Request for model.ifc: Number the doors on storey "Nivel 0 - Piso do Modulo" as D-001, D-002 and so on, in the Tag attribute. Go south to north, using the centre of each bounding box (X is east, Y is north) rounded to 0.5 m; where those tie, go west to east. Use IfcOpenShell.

First a look at what the model holds.

```python
import ifcopenshell
import ifcopenshell.util.element
import ifcopenshell.util.placement

model = ifcopenshell.open("model.ifc")
print(model.schema)
storey = next(s for s in model.by_type("IfcBuildingStorey") if s.Name == "Nivel 0 - Piso do Modulo")
doors = [e for e in ifcopenshell.util.element.get_decomposition(storey) if e.is_a("IfcDoor")]
for e in sorted(doors, key=lambda e: e.id()):
    origin = ifcopenshell.util.placement.get_local_placement(e.ObjectPlacement)[:3, 3]
    print(e.id(), e.Tag, e.Name, origin.round(2) + 0.0, sep=" | ")
```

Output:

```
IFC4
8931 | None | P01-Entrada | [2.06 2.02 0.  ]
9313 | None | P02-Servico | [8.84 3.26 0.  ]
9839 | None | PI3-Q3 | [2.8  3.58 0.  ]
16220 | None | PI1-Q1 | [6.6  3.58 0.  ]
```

```python
import ifcopenshell
import ifcopenshell.geom
import ifcopenshell.util.element
import ifcopenshell.util.shape

model = ifcopenshell.open("model.ifc")
settings = ifcopenshell.geom.settings()
settings.set("use-world-coords", True)


def centre(element):
    shape = ifcopenshell.geom.create_shape(settings, element)
    return ifcopenshell.util.shape.get_bbox_centroid(shape.geometry)


storey = next(s for s in model.by_type("IfcBuildingStorey") if s.Name == "Nivel 0 - Piso do Modulo")
doors = [e for e in ifcopenshell.util.element.get_decomposition(storey) if e.is_a("IfcDoor")]

# Insertion points can sit at a corner or the storey origin, so sort by the geometry (in metres).
centres = {e: centre(e) for e in doors}
doors.sort(key=lambda e: (round(centres[e][1] / 0.5), centres[e][0]))

for i, e in enumerate(doors, start=1):
    number = f"D-0{i:02d}"
    e.Tag = number
    print(e.id(), number)

model.write("model_edited.ifc")
```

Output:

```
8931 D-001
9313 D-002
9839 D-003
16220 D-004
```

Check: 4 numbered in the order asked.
